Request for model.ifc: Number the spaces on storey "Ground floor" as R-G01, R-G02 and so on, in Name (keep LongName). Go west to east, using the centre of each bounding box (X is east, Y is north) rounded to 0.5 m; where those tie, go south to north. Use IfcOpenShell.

First a look at what the model holds.

```python
import ifcopenshell
import ifcopenshell.util.element
import ifcopenshell.util.placement

model = ifcopenshell.open("model.ifc")
print(model.schema)
storey = next(s for s in model.by_type("IfcBuildingStorey") if s.Name == "Ground floor")
spaces = [e for e in ifcopenshell.util.element.get_decomposition(storey) if e.is_a("IfcSpace")]
for e in sorted(spaces, key=lambda e: e.id()):
    origin = ifcopenshell.util.placement.get_local_placement(e.ObjectPlacement)[:3, 3]
    print(e.id(), e.Name, e.LongName, origin.round(2) + 0.0, sep=" | ")
```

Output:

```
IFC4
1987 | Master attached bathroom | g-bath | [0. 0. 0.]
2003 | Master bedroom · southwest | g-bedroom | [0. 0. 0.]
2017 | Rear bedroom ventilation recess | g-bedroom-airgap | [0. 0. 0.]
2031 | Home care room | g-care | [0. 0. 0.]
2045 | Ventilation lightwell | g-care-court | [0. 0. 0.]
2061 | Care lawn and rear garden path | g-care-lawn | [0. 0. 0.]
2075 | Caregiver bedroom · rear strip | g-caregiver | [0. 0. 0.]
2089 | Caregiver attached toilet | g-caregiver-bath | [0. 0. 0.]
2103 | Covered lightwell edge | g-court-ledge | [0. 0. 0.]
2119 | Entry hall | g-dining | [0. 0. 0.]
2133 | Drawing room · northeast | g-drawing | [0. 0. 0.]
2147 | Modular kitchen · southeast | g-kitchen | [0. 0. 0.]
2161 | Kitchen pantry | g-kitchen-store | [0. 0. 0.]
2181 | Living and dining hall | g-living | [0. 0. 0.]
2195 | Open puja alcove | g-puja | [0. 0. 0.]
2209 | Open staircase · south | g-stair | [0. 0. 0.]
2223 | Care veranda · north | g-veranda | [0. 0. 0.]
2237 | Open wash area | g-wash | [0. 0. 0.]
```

```python
import ifcopenshell
import ifcopenshell.geom
import ifcopenshell.util.element
import ifcopenshell.util.shape

model = ifcopenshell.open("model.ifc")
settings = ifcopenshell.geom.settings()
settings.set("use-world-coords", True)


def centre(element):
    shape = ifcopenshell.geom.create_shape(settings, element)
    return ifcopenshell.util.shape.get_bbox_centroid(shape.geometry)


storey = next(s for s in model.by_type("IfcBuildingStorey") if s.Name == "Ground floor")
spaces = [e for e in ifcopenshell.util.element.get_decomposition(storey) if e.is_a("IfcSpace")]

# Insertion points can sit at a corner or the storey origin, so sort by the geometry (in metres).
centres = {e: centre(e) for e in spaces}
spaces.sort(key=lambda e: (round(centres[e][0] / 0.5), centres[e][1]))

for i, e in enumerate(spaces, start=1):
    number = f"R-G{i:02d}"
    e.Name = number
    print(e.id(), number)

model.write("model_edited.ifc")
```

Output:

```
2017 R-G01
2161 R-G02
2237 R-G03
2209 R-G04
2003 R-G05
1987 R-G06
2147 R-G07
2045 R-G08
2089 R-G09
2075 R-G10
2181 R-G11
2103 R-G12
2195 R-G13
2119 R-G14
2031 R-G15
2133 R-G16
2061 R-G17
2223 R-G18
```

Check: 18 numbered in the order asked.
